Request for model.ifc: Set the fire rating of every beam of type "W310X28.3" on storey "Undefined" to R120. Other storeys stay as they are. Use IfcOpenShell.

First a look at what the model holds.

```python
import ifcopenshell
import ifcopenshell.util.element

model = ifcopenshell.open("model.ifc")
print(model.schema)
storey = next(s for s in model.by_type("IfcBuildingStorey") if s.Name == "Undefined")
beams = [e for e in ifcopenshell.util.element.get_decomposition(storey) if e.is_a("IfcBeam")]
seen = {}
for e in beams:
    element_type = ifcopenshell.util.element.get_type(e)
    key = (element_type.Name if element_type != e and element_type else None, ifcopenshell.util.element.get_pset(e, "Pset_BeamCommon", "FireRating"))
    seen[key] = seen.get(key, 0) + 1
for (name, value), count in sorted(seen.items(), key=str):
    print(count, "x", name, "|", value)
```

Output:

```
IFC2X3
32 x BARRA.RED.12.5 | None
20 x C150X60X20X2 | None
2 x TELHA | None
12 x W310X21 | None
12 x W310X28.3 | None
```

```python
import ifcopenshell
import ifcopenshell.api.pset
import ifcopenshell.util.element

model = ifcopenshell.open("model.ifc")

storey = next(s for s in model.by_type("IfcBuildingStorey") if s.Name == "Undefined")
beams = [e for e in ifcopenshell.util.element.get_decomposition(storey) if e.is_a("IfcBeam")]

count = 0
for e in beams:
    element_type = ifcopenshell.util.element.get_type(e)
    if element_type in (None, e) or element_type.Name != "W310X28.3":
        continue
    found = ifcopenshell.util.element.get_pset(e, "Pset_BeamCommon", should_inherit=False)
    if found:
        pset = model.by_id(found["id"])
        if len(ifcopenshell.util.element.get_elements_by_pset(pset)) > 1:
            pset = ifcopenshell.api.pset.unshare_pset(model, products=[e], pset=pset)[0]
    else:
        pset = ifcopenshell.api.pset.add_pset(model, product=e, name="Pset_BeamCommon")
    ifcopenshell.api.pset.edit_pset(model, pset=pset, properties={"FireRating": "R120"})
    count += 1

print(count, "beams updated")

model.write("model_v2.ifc")
```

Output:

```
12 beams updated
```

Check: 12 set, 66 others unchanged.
